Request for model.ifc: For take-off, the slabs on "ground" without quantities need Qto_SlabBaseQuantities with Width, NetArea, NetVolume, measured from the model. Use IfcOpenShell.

First a look at what the model holds.

```python
import ifcopenshell
import ifcopenshell.util.element
import ifcopenshell.util.unit

model = ifcopenshell.open("model.ifc")
print(model.schema)
for unit_type in ("LENGTHUNIT", "AREAUNIT", "VOLUMEUNIT"):
    print(unit_type, ifcopenshell.util.unit.calculate_unit_scale(model, unit_type))
storey = next(s for s in model.by_type("IfcBuildingStorey") if s.Name == "ground")
slabs = [e for e in ifcopenshell.util.element.get_decomposition(storey) if e.is_a("IfcSlab")]
for e in sorted(slabs, key=lambda e: e.id()):
    print(e.id(), e.is_a(), e.Name, list(ifcopenshell.util.element.get_psets(e, qtos_only=True)), sep=" | ")
```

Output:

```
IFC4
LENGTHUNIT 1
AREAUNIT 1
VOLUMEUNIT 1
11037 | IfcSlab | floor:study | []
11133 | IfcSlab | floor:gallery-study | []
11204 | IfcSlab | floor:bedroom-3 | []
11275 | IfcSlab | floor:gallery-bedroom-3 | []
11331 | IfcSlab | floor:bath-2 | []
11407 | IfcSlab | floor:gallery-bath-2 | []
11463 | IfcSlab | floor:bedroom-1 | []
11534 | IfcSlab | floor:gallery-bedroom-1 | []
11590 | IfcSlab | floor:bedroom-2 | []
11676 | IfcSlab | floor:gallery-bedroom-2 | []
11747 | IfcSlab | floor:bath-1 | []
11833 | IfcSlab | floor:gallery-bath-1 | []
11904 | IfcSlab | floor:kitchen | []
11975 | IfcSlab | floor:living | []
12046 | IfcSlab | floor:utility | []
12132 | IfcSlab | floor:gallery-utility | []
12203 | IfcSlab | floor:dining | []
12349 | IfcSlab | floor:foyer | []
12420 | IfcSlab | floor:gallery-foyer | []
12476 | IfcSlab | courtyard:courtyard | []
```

```python
import ifcopenshell
import ifcopenshell.api.pset
import ifcopenshell.geom
import ifcopenshell.util.element
import ifcopenshell.util.shape
import ifcopenshell.util.unit

model = ifcopenshell.open("model.ifc")
unit_scale = ifcopenshell.util.unit.calculate_unit_scale(model)
area_scale = ifcopenshell.util.unit.calculate_unit_scale(model, "AREAUNIT")
volume_scale = ifcopenshell.util.unit.calculate_unit_scale(model, "VOLUMEUNIT")
settings = ifcopenshell.geom.settings()

storey = next(s for s in model.by_type("IfcBuildingStorey") if s.Name == "ground")
slabs = [e for e in ifcopenshell.util.element.get_decomposition(storey) if e.is_a("IfcSlab")]

for e in sorted(slabs, key=lambda e: e.id()):
    if ifcopenshell.util.element.get_psets(e, qtos_only=True, should_inherit=False):
        continue
    # Geometry comes back in metres, in the element's own axes.
    shape = ifcopenshell.geom.create_shape(settings, e)
    values = {
        "Width": ifcopenshell.util.shape.get_z(shape.geometry) / unit_scale,
        "NetArea": ifcopenshell.util.shape.get_footprint_area(shape.geometry) / area_scale,
        "NetVolume": ifcopenshell.util.shape.get_volume(shape.geometry) / volume_scale,
    }
    qto = ifcopenshell.api.pset.add_qto(model, product=e, name="Qto_SlabBaseQuantities")
    ifcopenshell.api.pset.edit_qto(model, qto=qto, properties=values)
    print(e.id(), {k: round(v, 3) for k, v in values.items()})

model.write("model_rev.ifc")
```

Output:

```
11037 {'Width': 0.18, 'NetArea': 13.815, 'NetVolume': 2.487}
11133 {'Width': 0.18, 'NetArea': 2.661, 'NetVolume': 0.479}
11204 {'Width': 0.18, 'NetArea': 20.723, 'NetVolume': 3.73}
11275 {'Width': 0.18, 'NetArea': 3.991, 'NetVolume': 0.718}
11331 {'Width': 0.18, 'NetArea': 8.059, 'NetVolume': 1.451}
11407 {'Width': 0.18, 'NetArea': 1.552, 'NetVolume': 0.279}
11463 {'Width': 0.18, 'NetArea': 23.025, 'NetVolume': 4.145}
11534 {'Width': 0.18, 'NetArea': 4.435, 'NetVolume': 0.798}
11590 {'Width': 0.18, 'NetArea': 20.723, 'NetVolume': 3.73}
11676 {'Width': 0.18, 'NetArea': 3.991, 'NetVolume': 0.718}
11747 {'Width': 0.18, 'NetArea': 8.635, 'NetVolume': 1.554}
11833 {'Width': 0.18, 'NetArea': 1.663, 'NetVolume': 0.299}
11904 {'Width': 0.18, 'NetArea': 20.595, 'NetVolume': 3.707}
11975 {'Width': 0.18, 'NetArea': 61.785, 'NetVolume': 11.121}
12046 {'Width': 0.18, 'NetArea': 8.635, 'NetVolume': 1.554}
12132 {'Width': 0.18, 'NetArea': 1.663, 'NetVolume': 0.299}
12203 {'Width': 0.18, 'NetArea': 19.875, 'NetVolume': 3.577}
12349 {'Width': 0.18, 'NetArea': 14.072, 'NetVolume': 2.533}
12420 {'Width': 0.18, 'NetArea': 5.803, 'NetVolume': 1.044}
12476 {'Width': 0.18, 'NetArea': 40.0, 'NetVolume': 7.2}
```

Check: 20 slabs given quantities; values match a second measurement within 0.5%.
